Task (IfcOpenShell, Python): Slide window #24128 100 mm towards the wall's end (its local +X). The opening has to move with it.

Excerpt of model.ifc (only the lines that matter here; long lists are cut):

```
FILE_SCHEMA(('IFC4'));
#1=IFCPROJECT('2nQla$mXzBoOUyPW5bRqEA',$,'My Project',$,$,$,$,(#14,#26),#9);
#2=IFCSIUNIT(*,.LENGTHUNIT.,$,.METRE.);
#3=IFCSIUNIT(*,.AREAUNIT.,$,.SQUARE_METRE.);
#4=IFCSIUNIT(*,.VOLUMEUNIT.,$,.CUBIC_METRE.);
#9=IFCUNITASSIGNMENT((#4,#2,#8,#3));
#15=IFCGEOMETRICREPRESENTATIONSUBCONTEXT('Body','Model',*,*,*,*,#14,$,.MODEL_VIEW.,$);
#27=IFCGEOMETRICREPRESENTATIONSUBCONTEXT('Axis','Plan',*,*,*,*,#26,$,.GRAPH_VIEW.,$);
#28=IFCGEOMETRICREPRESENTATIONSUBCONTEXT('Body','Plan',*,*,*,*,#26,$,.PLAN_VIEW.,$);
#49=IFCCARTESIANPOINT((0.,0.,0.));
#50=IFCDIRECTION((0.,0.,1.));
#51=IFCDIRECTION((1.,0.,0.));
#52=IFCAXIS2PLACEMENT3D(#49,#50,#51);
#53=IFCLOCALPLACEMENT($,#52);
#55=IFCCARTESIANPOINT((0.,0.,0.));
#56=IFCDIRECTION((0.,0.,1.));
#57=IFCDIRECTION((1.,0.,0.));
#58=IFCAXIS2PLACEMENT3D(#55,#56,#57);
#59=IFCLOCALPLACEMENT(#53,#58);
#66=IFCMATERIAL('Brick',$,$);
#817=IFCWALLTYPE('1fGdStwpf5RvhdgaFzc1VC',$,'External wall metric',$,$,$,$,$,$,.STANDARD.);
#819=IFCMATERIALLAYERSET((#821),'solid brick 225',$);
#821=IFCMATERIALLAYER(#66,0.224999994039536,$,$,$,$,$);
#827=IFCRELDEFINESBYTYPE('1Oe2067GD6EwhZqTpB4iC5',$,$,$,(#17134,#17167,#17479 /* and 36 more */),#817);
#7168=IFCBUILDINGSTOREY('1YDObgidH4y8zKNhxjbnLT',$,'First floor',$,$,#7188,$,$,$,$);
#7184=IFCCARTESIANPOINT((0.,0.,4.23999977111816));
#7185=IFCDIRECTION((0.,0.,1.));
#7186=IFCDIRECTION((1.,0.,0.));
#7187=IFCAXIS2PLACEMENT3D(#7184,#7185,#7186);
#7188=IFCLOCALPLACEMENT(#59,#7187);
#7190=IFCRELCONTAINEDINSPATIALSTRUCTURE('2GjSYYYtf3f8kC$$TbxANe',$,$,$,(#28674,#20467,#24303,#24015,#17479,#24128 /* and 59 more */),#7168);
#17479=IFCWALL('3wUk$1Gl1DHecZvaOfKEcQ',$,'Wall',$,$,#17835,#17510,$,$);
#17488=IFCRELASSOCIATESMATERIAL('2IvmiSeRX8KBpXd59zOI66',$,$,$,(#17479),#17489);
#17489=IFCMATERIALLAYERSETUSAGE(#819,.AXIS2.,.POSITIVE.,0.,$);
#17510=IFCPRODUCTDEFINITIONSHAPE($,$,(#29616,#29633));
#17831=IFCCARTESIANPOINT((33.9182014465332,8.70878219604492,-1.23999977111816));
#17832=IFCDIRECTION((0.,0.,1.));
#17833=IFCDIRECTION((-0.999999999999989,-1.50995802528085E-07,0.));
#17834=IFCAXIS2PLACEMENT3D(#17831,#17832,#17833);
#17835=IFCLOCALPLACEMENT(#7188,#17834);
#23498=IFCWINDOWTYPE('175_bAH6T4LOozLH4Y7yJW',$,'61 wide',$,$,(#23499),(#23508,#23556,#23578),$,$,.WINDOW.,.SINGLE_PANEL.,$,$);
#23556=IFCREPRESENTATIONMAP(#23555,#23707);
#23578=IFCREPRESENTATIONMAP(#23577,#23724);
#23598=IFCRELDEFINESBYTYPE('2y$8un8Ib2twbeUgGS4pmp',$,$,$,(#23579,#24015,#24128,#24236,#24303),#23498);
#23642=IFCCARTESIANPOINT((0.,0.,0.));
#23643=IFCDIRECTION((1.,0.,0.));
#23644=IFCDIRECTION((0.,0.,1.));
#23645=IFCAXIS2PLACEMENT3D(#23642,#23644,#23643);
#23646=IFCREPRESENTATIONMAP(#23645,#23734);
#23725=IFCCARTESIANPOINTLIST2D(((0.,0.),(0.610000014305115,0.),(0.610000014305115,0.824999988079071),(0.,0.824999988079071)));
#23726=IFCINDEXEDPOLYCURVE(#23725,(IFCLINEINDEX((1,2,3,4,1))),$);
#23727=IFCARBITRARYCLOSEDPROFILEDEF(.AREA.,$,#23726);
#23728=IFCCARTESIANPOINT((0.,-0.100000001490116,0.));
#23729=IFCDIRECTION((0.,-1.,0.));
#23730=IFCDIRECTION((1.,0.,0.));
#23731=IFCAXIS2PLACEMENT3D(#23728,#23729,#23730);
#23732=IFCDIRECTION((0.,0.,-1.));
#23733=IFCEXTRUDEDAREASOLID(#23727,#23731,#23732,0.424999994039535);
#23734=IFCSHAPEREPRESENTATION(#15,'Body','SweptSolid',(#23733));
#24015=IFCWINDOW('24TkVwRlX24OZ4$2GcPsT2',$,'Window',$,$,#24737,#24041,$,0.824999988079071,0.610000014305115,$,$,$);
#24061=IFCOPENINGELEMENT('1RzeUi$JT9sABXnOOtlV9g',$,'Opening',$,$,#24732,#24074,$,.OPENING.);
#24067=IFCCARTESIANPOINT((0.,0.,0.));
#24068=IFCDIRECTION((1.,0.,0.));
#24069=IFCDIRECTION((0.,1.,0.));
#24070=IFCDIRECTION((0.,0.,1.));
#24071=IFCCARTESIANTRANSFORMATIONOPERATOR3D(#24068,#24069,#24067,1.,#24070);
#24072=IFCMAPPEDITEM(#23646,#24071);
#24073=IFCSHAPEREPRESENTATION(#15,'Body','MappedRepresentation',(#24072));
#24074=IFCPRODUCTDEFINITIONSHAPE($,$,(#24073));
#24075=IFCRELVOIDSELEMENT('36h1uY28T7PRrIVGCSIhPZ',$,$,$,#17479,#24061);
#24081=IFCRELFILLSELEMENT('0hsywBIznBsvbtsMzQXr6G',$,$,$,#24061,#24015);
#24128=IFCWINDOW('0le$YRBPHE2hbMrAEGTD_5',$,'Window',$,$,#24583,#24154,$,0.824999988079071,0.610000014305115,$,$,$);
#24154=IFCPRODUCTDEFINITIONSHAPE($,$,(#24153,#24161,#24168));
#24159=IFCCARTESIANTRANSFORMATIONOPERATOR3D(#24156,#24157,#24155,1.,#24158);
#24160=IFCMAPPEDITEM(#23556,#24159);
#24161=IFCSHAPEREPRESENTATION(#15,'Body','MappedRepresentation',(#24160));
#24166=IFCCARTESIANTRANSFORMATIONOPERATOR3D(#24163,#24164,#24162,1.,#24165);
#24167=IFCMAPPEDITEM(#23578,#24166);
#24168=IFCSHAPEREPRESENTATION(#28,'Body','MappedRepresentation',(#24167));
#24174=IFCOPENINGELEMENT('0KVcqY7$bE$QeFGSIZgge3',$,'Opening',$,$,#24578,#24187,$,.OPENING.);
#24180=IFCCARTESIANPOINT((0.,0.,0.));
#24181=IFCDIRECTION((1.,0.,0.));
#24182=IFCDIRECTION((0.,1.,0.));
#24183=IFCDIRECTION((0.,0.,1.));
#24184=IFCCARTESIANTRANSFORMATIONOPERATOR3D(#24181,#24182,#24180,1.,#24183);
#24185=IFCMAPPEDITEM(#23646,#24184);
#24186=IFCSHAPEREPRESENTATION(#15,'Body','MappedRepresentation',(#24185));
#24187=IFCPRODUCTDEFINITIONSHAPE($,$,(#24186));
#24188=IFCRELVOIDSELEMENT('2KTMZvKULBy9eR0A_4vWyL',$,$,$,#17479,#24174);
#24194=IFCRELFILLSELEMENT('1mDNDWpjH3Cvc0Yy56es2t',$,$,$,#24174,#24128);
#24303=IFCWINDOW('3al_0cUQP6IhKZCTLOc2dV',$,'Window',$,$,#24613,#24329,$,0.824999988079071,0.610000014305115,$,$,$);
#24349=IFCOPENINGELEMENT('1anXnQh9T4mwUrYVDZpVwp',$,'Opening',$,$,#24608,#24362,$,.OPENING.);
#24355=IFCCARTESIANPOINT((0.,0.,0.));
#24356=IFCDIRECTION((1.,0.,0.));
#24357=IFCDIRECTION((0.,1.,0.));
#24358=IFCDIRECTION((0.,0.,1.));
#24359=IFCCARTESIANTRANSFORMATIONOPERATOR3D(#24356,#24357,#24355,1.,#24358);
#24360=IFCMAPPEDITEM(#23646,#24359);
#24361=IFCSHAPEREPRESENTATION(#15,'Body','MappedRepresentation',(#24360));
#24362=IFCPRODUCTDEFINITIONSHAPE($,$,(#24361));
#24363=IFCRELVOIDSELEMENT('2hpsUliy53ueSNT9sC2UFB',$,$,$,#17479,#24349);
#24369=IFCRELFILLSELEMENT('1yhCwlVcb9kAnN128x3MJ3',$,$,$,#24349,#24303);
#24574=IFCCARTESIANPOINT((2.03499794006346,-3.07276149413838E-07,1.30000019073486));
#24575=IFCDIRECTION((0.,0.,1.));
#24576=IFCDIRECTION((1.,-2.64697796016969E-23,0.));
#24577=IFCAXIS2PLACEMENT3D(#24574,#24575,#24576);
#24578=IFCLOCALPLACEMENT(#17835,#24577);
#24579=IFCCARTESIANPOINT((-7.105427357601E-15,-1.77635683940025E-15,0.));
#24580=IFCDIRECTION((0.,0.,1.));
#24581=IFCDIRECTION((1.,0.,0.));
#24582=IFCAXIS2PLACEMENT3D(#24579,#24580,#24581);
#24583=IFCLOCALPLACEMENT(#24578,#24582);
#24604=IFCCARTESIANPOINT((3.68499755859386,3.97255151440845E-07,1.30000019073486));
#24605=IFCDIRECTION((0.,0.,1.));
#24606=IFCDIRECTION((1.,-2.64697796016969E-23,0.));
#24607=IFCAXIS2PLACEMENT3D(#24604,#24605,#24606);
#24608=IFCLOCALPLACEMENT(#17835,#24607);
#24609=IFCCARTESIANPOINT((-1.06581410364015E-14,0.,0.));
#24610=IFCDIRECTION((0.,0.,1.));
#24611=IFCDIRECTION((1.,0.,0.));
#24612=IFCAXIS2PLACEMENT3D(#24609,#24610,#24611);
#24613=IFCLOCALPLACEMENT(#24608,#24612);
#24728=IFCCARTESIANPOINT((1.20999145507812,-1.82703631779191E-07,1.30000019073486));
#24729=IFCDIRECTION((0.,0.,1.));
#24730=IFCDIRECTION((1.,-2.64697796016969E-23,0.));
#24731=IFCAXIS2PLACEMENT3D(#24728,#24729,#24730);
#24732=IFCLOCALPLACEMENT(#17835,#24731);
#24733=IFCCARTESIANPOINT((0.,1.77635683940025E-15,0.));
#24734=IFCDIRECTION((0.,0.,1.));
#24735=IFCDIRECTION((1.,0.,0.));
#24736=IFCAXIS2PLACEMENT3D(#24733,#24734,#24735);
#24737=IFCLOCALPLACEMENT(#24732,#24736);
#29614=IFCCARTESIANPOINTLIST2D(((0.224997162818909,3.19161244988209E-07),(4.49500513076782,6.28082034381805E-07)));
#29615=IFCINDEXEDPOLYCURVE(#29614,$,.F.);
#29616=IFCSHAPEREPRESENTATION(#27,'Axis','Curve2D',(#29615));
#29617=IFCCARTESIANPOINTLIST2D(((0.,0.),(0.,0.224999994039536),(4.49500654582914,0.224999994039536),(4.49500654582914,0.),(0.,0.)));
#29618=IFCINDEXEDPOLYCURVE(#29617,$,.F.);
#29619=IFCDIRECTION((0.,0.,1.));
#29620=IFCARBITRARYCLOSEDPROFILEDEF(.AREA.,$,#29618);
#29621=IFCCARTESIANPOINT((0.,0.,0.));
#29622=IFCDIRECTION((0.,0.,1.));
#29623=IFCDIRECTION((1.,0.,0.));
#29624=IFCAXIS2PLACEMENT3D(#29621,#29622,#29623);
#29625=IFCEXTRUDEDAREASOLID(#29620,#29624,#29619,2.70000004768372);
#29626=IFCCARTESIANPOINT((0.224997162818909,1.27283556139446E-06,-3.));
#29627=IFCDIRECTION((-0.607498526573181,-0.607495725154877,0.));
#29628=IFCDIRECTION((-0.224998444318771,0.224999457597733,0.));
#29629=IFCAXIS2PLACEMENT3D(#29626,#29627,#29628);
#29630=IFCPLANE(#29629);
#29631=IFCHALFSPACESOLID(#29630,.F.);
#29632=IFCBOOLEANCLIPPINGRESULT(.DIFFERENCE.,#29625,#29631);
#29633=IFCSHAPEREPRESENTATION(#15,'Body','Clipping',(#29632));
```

```python
import ifcopenshell
import ifcopenshell.api.geometry
import ifcopenshell.util.placement
import ifcopenshell.util.unit

model = ifcopenshell.open("model.ifc")
unit_scale = ifcopenshell.util.unit.calculate_unit_scale(model)

window = model.by_guid("0le$YRBPHE2hbMrAEGTD_5")
opening = window.FillsVoids[0].RelatingOpeningElement
wall = opening.VoidsElements[0].RelatingBuildingElement

wall_matrix = ifcopenshell.util.placement.get_local_placement(wall.ObjectPlacement)
shift = wall_matrix[:3, 0] * 0.1 / unit_scale
before = ifcopenshell.util.placement.get_local_placement(window.ObjectPlacement)[:3, 3].copy()

# The window is placed relative to its opening, so it follows when the opening moves.
matrix = ifcopenshell.util.placement.get_local_placement(opening.ObjectPlacement)
matrix[:3, 3] += shift
ifcopenshell.api.geometry.edit_object_placement(
    model, product=opening, matrix=matrix, is_si=False, should_transform_children=True
)

after = ifcopenshell.util.placement.get_local_placement(window.ObjectPlacement)[:3, 3]
print("window moved by", (after - before).round(3) + 0.0)

model.write("model_rev.ifc")
```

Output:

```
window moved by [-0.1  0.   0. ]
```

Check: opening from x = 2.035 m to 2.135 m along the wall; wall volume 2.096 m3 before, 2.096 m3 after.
